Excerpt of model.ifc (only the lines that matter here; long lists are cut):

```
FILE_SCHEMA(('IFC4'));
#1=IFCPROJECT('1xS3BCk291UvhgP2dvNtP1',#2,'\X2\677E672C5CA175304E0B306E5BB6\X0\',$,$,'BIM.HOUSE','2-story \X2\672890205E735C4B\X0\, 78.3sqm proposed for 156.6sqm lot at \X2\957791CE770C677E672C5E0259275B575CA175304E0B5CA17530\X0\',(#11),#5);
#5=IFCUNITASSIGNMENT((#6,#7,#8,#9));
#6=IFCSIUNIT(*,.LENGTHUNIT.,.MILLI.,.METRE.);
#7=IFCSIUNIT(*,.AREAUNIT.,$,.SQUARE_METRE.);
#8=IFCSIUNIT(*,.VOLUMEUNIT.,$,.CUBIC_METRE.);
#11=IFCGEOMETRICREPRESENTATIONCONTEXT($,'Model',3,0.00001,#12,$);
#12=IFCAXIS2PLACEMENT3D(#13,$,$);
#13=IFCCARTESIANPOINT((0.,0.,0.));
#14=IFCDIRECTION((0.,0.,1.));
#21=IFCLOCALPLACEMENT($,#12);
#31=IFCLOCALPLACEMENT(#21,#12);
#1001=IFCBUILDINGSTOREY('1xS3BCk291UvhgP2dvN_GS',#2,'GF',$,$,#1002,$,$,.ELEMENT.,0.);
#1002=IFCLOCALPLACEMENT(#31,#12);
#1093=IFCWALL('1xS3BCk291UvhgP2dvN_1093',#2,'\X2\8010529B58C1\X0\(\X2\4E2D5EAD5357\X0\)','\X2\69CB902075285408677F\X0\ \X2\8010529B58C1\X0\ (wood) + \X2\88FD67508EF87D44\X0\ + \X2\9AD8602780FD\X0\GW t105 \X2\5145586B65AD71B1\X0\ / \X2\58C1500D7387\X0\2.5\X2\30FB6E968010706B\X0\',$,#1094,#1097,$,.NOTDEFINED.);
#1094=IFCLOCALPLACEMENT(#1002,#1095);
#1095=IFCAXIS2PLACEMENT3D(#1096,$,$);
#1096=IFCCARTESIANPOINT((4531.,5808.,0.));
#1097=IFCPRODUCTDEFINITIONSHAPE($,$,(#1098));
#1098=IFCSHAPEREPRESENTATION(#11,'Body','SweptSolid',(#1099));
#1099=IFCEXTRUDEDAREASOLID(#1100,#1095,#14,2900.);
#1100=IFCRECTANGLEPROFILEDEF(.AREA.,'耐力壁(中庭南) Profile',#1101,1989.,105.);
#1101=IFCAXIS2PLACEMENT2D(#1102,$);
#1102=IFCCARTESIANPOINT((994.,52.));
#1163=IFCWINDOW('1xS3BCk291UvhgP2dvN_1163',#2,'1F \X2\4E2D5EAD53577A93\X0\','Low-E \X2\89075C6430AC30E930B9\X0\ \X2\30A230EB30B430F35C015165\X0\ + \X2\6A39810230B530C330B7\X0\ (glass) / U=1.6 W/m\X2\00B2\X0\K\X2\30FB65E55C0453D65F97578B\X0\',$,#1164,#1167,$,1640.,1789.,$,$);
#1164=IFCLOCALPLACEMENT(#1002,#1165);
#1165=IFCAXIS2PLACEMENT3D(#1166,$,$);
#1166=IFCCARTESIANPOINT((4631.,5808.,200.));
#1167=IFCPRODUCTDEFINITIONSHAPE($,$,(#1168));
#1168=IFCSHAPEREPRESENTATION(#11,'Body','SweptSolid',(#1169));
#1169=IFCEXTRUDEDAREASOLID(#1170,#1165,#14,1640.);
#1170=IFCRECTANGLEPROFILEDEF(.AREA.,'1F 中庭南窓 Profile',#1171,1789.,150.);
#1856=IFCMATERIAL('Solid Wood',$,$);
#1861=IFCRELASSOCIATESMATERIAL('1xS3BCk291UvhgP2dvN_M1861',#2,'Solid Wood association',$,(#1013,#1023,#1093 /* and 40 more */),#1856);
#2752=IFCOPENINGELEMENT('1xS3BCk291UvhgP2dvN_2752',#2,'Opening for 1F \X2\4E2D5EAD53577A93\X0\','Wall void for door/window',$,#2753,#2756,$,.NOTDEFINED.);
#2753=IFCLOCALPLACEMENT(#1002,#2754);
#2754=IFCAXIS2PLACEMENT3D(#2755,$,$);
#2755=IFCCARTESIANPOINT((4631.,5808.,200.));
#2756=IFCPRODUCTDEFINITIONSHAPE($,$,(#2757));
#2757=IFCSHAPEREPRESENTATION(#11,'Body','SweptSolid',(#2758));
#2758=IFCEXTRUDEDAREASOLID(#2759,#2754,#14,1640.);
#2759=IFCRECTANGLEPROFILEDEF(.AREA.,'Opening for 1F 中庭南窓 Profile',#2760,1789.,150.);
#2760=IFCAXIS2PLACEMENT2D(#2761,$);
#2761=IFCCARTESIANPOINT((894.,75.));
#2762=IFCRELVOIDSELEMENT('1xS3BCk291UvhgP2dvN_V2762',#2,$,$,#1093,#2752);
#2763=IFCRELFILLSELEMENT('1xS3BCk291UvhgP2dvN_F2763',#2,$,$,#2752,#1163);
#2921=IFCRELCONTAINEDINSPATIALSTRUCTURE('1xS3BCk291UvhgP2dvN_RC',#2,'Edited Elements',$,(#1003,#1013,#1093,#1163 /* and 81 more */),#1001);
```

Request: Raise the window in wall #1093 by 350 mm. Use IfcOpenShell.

```python
import numpy as np
import ifcopenshell
import ifcopenshell.api.geometry
import ifcopenshell.util.placement
import ifcopenshell.util.unit

model = ifcopenshell.open("model.ifc")
unit_scale = ifcopenshell.util.unit.calculate_unit_scale(model)

window = model.by_guid("1xS3BCk291UvhgP2dvN_1163")
opening = window.FillsVoids[0].RelatingOpeningElement
dz = 0.35 / unit_scale

shift = np.array([0.0, 0.0, dz])
# The window is not placed relative to its opening, so move both.
for product in (opening, window):
    matrix = ifcopenshell.util.placement.get_local_placement(product.ObjectPlacement)
    matrix[:3, 3] += shift
    ifcopenshell.api.geometry.edit_object_placement(model, product=product, matrix=matrix, is_si=False)

print(f"moved by {dz * unit_scale:+.3f} m")

model.write("model-out.ifc")
```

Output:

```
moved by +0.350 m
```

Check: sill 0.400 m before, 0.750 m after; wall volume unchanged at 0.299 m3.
